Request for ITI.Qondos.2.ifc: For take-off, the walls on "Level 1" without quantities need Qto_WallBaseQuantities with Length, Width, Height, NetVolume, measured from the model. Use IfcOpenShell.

First a look at what the model holds.

```python
import ifcopenshell
import ifcopenshell.util.element
import ifcopenshell.util.unit

model = ifcopenshell.open("ITI.Qondos.2.ifc")
print(model.schema)
for unit_type in ("LENGTHUNIT", "AREAUNIT", "VOLUMEUNIT"):
    print(unit_type, ifcopenshell.util.unit.calculate_unit_scale(model, unit_type))
storey = next(s for s in model.by_type("IfcBuildingStorey") if s.Name == "Level 1")
walls = [e for e in ifcopenshell.util.element.get_decomposition(storey) if e.is_a("IfcWall")]
for e in sorted(walls, key=lambda e: e.id()):
    print(e.id(), e.is_a(), e.Name, list(ifcopenshell.util.element.get_psets(e, qtos_only=True)), sep=" | ")
```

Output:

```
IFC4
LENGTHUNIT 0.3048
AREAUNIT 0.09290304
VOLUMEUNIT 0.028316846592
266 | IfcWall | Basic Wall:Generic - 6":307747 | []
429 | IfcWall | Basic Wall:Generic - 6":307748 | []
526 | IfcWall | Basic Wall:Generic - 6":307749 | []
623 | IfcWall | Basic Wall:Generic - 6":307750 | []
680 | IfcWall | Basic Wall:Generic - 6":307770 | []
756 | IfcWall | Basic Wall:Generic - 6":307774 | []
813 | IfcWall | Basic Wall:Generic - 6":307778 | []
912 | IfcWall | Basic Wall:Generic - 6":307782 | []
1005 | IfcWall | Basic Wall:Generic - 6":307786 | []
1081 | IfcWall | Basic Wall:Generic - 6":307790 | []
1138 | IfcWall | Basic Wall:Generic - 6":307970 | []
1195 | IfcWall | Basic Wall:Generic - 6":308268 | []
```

```python
import ifcopenshell
import ifcopenshell.api.pset
import ifcopenshell.geom
import ifcopenshell.util.element
import ifcopenshell.util.shape
import ifcopenshell.util.unit

model = ifcopenshell.open("ITI.Qondos.2.ifc")
unit_scale = ifcopenshell.util.unit.calculate_unit_scale(model)
volume_scale = ifcopenshell.util.unit.calculate_unit_scale(model, "VOLUMEUNIT")
settings = ifcopenshell.geom.settings()

storey = next(s for s in model.by_type("IfcBuildingStorey") if s.Name == "Level 1")
walls = [e for e in ifcopenshell.util.element.get_decomposition(storey) if e.is_a("IfcWall")]

for e in sorted(walls, key=lambda e: e.id()):
    if ifcopenshell.util.element.get_psets(e, qtos_only=True, should_inherit=False):
        continue
    # Geometry comes back in metres, in the element's own axes.
    shape = ifcopenshell.geom.create_shape(settings, e)
    values = {
        "Length": ifcopenshell.util.shape.get_x(shape.geometry) / unit_scale,
        "Width": ifcopenshell.util.shape.get_y(shape.geometry) / unit_scale,
        "Height": ifcopenshell.util.shape.get_z(shape.geometry) / unit_scale,
        "NetVolume": ifcopenshell.util.shape.get_volume(shape.geometry) / volume_scale,
    }
    qto = ifcopenshell.api.pset.add_qto(model, product=e, name="Qto_WallBaseQuantities")
    ifcopenshell.api.pset.edit_qto(model, qto=qto, properties=values)
    print(e.id(), {k: round(v, 3) for k, v in values.items()})

model.write("ITI.Qondos.2_rev.ifc")
```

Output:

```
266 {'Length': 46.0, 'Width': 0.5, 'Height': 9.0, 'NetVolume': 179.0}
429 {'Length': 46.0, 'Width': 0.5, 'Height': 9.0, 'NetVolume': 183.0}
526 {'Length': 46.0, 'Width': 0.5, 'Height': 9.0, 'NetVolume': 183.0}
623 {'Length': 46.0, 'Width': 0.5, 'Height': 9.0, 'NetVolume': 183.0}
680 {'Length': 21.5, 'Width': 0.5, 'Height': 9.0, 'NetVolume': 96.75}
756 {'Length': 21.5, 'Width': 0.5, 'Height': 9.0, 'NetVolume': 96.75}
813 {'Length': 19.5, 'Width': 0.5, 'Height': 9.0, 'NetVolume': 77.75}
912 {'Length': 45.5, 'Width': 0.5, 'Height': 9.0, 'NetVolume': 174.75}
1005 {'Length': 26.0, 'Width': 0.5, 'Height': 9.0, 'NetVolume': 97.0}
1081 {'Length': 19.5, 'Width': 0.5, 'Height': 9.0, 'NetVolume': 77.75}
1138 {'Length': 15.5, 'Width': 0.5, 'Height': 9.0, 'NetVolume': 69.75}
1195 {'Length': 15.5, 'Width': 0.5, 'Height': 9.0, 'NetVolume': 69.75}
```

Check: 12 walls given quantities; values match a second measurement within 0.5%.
